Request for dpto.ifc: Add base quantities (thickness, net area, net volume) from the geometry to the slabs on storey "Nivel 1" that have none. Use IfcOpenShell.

First a look at what the model holds.

```python
import ifcopenshell
import ifcopenshell.util.element
import ifcopenshell.util.unit

model = ifcopenshell.open("dpto.ifc")
print(model.schema)
for unit_type in ("LENGTHUNIT", "AREAUNIT", "VOLUMEUNIT"):
    print(unit_type, ifcopenshell.util.unit.calculate_unit_scale(model, unit_type))
storey = next(s for s in model.by_type("IfcBuildingStorey") if s.Name == "Nivel 1")
slabs = [e for e in ifcopenshell.util.element.get_decomposition(storey) if e.is_a("IfcSlab")]
for e in sorted(slabs, key=lambda e: e.id()):
    print(e.id(), e.is_a(), e.Name, list(ifcopenshell.util.element.get_psets(e, qtos_only=True)), sep=" | ")
```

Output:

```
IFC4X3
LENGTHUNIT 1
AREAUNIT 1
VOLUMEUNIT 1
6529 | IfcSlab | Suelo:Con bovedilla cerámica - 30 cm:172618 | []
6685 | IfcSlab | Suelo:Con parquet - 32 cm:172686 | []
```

```python
import ifcopenshell
import ifcopenshell.api.pset
import ifcopenshell.geom
import ifcopenshell.util.element
import ifcopenshell.util.shape
import ifcopenshell.util.unit

model = ifcopenshell.open("dpto.ifc")
unit_scale = ifcopenshell.util.unit.calculate_unit_scale(model)
area_scale = ifcopenshell.util.unit.calculate_unit_scale(model, "AREAUNIT")
volume_scale = ifcopenshell.util.unit.calculate_unit_scale(model, "VOLUMEUNIT")
settings = ifcopenshell.geom.settings()

storey = next(s for s in model.by_type("IfcBuildingStorey") if s.Name == "Nivel 1")
slabs = [e for e in ifcopenshell.util.element.get_decomposition(storey) if e.is_a("IfcSlab")]

for e in sorted(slabs, key=lambda e: e.id()):
    if ifcopenshell.util.element.get_psets(e, qtos_only=True, should_inherit=False):
        continue
    # Geometry comes back in metres, in the element's own axes.
    shape = ifcopenshell.geom.create_shape(settings, e)
    values = {
        "Width": ifcopenshell.util.shape.get_z(shape.geometry) / unit_scale,
        "NetArea": ifcopenshell.util.shape.get_footprint_area(shape.geometry) / area_scale,
        "NetVolume": ifcopenshell.util.shape.get_volume(shape.geometry) / volume_scale,
    }
    qto = ifcopenshell.api.pset.add_qto(model, product=e, name="Qto_SlabBaseQuantities")
    ifcopenshell.api.pset.edit_qto(model, qto=qto, properties=values)
    print(e.id(), {k: round(v, 3) for k, v in values.items()})

model.write("dpto_v2.ifc")
```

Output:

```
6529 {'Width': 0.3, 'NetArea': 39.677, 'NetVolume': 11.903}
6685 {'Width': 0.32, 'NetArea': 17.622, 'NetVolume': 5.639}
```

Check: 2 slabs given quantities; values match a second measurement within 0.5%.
